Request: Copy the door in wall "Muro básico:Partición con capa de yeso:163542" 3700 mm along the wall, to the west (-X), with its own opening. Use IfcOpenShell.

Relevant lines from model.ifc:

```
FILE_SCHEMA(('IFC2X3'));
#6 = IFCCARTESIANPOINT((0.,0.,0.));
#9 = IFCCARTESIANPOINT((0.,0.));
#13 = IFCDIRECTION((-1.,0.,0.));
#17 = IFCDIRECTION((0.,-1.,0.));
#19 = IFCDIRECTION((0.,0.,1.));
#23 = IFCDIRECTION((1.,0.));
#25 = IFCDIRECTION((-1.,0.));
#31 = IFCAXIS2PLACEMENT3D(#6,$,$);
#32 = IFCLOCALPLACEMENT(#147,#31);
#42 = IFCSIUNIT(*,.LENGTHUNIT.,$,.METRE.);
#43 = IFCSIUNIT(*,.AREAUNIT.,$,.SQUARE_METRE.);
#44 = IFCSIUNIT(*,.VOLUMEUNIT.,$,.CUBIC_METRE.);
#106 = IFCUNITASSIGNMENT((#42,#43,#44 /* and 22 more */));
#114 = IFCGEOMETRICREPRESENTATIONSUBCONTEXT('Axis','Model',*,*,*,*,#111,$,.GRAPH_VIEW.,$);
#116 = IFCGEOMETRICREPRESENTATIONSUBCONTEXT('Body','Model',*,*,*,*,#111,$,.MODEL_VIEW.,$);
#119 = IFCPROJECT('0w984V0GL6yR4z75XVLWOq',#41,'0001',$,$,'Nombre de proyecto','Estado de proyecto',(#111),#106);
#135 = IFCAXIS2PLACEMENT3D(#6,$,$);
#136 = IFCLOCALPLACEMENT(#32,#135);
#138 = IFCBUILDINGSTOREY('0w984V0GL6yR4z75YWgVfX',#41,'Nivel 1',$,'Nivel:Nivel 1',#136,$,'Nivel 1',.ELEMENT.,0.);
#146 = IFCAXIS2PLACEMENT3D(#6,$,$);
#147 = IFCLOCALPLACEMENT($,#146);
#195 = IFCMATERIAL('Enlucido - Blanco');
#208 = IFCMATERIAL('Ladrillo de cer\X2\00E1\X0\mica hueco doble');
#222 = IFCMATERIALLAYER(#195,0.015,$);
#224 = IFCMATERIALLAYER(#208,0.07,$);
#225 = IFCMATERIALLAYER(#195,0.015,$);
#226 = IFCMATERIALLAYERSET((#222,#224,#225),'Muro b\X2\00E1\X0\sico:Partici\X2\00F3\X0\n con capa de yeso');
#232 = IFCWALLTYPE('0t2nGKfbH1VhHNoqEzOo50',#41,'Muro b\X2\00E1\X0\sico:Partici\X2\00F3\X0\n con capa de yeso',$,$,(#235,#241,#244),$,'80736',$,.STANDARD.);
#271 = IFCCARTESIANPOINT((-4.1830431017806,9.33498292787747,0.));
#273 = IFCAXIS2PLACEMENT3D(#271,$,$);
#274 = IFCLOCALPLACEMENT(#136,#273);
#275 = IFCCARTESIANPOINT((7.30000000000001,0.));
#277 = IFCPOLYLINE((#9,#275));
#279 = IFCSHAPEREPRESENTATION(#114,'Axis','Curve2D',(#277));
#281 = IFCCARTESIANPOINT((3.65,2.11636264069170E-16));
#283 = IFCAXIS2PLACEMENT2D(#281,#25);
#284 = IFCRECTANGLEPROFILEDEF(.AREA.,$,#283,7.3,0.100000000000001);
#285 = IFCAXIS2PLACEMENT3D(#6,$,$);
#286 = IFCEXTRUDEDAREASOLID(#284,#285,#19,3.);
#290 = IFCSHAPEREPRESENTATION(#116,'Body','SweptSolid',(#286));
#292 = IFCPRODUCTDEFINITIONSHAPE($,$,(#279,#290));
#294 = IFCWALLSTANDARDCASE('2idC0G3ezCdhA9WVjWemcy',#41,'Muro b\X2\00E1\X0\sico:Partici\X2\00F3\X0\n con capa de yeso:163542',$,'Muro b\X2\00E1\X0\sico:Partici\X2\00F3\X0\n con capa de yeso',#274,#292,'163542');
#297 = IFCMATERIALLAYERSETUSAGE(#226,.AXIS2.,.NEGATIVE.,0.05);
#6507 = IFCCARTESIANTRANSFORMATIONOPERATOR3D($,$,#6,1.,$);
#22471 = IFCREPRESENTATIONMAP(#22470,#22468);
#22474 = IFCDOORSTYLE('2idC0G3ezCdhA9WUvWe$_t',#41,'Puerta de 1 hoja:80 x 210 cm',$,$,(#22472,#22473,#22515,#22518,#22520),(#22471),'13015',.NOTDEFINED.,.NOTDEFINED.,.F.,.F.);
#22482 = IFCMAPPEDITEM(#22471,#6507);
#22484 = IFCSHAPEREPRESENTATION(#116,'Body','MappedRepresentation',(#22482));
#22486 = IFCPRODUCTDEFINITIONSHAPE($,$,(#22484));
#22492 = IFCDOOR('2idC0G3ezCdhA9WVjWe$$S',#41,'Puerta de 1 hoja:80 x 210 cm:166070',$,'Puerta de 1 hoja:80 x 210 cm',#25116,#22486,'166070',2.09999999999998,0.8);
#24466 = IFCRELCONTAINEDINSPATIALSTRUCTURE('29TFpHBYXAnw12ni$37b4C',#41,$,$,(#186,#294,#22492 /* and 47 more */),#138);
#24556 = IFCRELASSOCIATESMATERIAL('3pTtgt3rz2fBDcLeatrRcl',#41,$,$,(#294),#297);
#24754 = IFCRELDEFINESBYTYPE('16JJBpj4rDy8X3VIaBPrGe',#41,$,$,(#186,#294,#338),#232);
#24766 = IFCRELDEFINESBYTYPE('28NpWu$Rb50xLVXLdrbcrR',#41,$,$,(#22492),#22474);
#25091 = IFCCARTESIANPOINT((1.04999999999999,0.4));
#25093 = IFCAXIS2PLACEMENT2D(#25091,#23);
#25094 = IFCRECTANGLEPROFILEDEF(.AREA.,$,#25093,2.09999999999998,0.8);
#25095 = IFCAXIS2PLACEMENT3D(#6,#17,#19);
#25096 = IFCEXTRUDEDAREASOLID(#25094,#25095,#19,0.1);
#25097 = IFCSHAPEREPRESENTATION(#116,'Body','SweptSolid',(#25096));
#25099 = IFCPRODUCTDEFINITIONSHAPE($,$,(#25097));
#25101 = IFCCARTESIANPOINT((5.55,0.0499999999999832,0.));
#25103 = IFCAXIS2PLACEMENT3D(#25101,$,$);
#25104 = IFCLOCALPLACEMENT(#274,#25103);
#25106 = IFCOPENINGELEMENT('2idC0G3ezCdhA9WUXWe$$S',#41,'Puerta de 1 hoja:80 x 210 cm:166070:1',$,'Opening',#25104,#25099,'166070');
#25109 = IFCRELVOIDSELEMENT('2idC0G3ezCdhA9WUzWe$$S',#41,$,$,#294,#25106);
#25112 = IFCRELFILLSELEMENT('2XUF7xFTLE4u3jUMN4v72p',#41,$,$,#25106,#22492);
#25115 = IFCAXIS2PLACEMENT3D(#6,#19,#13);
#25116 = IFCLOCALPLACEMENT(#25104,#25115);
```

```python
import ifcopenshell
import ifcopenshell.api.feature
import ifcopenshell.api.geometry
import ifcopenshell.api.root
import ifcopenshell.geom
import ifcopenshell.util.element
import ifcopenshell.util.placement
import ifcopenshell.util.shape

model = ifcopenshell.open("model.ifc")
settings = ifcopenshell.geom.settings()


def volume(element):
    """Net volume in cubic metres, openings subtracted."""
    shape = ifcopenshell.geom.create_shape(settings, element)
    return ifcopenshell.util.shape.get_volume(shape.geometry)


def reuse_history(source, copy):
    """copy_class also copies each property set's owner history, people and application; keep the originals."""
    for rel in copy.IsDefinedBy:
        if rel.is_a("IfcRelDefinesByProperties") and (history := rel.RelatingPropertyDefinition.OwnerHistory):
            rel.RelatingPropertyDefinition.OwnerHistory = source.OwnerHistory
            ifcopenshell.util.element.remove_deep2(model, history)


door = model.by_id(22492)
opening = door.FillsVoids[0].RelatingOpeningElement
wall = opening.VoidsElements[0].RelatingBuildingElement
before = volume(wall)
shift = ifcopenshell.util.placement.get_local_placement(wall.ObjectPlacement)[:3, 0] * -3.7

# copy_class copies the void relationship, type, container and properties, but no geometry.
new_opening = ifcopenshell.api.root.copy_class(model, product=opening)
new_opening.Representation = ifcopenshell.util.element.copy_deep(
    model, opening.Representation, exclude=["IfcGeometricRepresentationContext", "IfcRepresentationMap"]
)
new_opening.Name = "Puerta de 1 hoja:80 x 210 cm"
new_opening.Tag = None
new_door = ifcopenshell.api.root.copy_class(model, product=door)
new_door.Representation = ifcopenshell.util.element.copy_deep(
    model, door.Representation, exclude=["IfcGeometricRepresentationContext", "IfcRepresentationMap"]
)
new_door.Name = "Puerta de 1 hoja:80 x 210 cm"
new_door.Tag = None
reuse_history(door, new_door)
fills = ifcopenshell.api.feature.add_filling(model, opening=new_opening, element=new_door)
fills.OwnerHistory = new_door.OwnerHistory  # required in IFC2X3

for old, new in ((opening, new_opening), (door, new_door)):
    matrix = ifcopenshell.util.placement.get_local_placement(old.ObjectPlacement)
    matrix[:3, 3] += shift
    ifcopenshell.api.geometry.edit_object_placement(model, product=new, matrix=matrix, is_si=False)

after = volume(wall)

print(f"wall volume {before:.3f} -> {after:.3f} m3")

model.write("model_rev.ifc")
```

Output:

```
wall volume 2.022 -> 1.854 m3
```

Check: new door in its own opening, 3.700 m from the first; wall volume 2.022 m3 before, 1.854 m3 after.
